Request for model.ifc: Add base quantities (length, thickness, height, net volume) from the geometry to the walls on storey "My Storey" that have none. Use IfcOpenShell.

First a look at what the model holds.

```python
import ifcopenshell
import ifcopenshell.util.element
import ifcopenshell.util.unit

model = ifcopenshell.open("model.ifc")
print(model.schema)
for unit_type in ("LENGTHUNIT", "AREAUNIT", "VOLUMEUNIT"):
    print(unit_type, ifcopenshell.util.unit.calculate_unit_scale(model, unit_type))
storey = next(s for s in model.by_type("IfcBuildingStorey") if s.Name == "My Storey")
walls = [e for e in ifcopenshell.util.element.get_decomposition(storey) if e.is_a("IfcWall")]
for e in sorted(walls, key=lambda e: e.id()):
    print(e.id(), e.is_a(), e.Name, list(ifcopenshell.util.element.get_psets(e, qtos_only=True)), sep=" | ")
```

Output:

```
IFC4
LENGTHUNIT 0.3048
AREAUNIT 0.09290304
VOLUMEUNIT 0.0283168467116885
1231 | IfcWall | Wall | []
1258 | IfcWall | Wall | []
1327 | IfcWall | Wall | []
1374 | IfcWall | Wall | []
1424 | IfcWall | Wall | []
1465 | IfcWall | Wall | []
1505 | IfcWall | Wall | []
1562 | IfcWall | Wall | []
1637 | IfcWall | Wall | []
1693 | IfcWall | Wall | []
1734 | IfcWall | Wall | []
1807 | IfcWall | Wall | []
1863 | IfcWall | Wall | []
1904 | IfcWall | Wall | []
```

```python
import ifcopenshell
import ifcopenshell.api.pset
import ifcopenshell.geom
import ifcopenshell.util.element
import ifcopenshell.util.shape
import ifcopenshell.util.unit

model = ifcopenshell.open("model.ifc")
unit_scale = ifcopenshell.util.unit.calculate_unit_scale(model)
volume_scale = ifcopenshell.util.unit.calculate_unit_scale(model, "VOLUMEUNIT")
settings = ifcopenshell.geom.settings()

storey = next(s for s in model.by_type("IfcBuildingStorey") if s.Name == "My Storey")
walls = [e for e in ifcopenshell.util.element.get_decomposition(storey) if e.is_a("IfcWall")]

for e in sorted(walls, key=lambda e: e.id()):
    if ifcopenshell.util.element.get_psets(e, qtos_only=True, should_inherit=False):
        continue
    # Geometry comes back in metres, in the element's own axes.
    shape = ifcopenshell.geom.create_shape(settings, e)
    values = {
        "Length": ifcopenshell.util.shape.get_x(shape.geometry) / unit_scale,
        "Width": ifcopenshell.util.shape.get_y(shape.geometry) / unit_scale,
        "Height": ifcopenshell.util.shape.get_z(shape.geometry) / unit_scale,
        "NetVolume": ifcopenshell.util.shape.get_volume(shape.geometry) / volume_scale,
    }
    qto = ifcopenshell.api.pset.add_qto(model, product=e, name="Qto_WallBaseQuantities")
    ifcopenshell.api.pset.edit_qto(model, qto=qto, properties=values)
    print(e.id(), {k: round(v, 3) for k, v in values.items()})

model.write("model_v2.ifc")
```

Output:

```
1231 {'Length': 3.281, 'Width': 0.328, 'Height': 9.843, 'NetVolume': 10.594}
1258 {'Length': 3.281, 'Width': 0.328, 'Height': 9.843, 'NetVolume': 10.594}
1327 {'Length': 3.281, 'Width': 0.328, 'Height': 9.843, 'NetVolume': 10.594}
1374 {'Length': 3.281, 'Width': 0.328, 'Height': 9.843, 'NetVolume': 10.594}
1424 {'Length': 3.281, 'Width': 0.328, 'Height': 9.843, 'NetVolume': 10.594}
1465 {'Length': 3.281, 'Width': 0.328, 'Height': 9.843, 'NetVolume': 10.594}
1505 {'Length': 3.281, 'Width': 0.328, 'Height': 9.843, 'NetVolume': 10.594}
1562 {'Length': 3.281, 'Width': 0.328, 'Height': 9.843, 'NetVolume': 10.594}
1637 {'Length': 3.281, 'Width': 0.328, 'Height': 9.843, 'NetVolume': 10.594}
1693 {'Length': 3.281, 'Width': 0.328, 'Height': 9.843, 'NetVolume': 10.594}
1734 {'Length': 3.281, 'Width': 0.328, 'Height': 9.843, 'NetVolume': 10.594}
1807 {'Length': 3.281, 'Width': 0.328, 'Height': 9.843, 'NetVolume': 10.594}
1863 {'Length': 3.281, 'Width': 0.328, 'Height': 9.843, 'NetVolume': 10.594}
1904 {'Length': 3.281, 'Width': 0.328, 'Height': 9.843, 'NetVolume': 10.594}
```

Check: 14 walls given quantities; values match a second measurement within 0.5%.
